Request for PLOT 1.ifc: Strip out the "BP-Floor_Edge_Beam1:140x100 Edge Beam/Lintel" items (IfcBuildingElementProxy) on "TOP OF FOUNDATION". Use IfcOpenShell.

First a look at what the model holds.

```python
import ifcopenshell
import ifcopenshell.util.element

model = ifcopenshell.open("PLOT 1.ifc")
print(model.schema)
storey = next(s for s in model.by_type("IfcBuildingStorey") if s.Name == "TOP OF FOUNDATION")
proxies = [e for e in ifcopenshell.util.element.get_decomposition(storey) if e.is_a("IfcBuildingElementProxy")]
seen = {}
for e in proxies:
    element_type = ifcopenshell.util.element.get_type(e)
    name = element_type.Name if element_type not in (None, e) else None
    seen[name] = seen.get(name, 0) + 1
for name, count in sorted(seen.items(), key=str):
    print(count, "x", name)
```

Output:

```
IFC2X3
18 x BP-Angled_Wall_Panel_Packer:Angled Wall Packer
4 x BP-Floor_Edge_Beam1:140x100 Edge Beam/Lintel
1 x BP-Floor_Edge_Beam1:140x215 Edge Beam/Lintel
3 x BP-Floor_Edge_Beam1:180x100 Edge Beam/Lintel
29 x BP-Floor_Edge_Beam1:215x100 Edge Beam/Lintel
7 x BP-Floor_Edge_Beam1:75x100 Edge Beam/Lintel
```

```python
import ifcopenshell
import ifcopenshell.api.root
import ifcopenshell.util.element

model = ifcopenshell.open("PLOT 1.ifc")

storey = next(s for s in model.by_type("IfcBuildingStorey") if s.Name == "TOP OF FOUNDATION")
proxies = [e for e in ifcopenshell.util.element.get_decomposition(storey) if e.is_a("IfcBuildingElementProxy")]
targets = [e for e in proxies if (t := ifcopenshell.util.element.get_type(e)) not in (None, e) and t.Name == "BP-Floor_Edge_Beam1:140x100 Edge Beam/Lintel"]

for e in targets:
    ifcopenshell.api.root.remove_product(model, product=e)
print(len(targets), "removed")

model.write("PLOT 1_v2.ifc")
```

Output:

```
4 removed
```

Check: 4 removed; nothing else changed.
